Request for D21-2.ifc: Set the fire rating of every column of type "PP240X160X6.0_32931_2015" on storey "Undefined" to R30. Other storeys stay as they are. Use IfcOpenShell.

First a look at what the model holds.

```python
import ifcopenshell
import ifcopenshell.util.element

model = ifcopenshell.open("D21-2.ifc")
print(model.schema)
storey = next(s for s in model.by_type("IfcBuildingStorey") if s.Name == "Undefined")
columns = [e for e in ifcopenshell.util.element.get_decomposition(storey) if e.is_a("IfcColumn")]
seen = {}
for e in columns:
    element_type = ifcopenshell.util.element.get_type(e)
    key = (element_type.Name if element_type != e and element_type else None, ifcopenshell.util.element.get_pset(e, "Pset_ColumnCommon", "FireRating"))
    seen[key] = seen.get(key, 0) + 1
for (name, value), count in sorted(seen.items(), key=str):
    print(count, "x", name, "|", value)
```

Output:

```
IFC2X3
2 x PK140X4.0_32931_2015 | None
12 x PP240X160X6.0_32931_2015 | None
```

```python
import ifcopenshell
import ifcopenshell.api.pset
import ifcopenshell.util.element

model = ifcopenshell.open("D21-2.ifc")

storey = next(s for s in model.by_type("IfcBuildingStorey") if s.Name == "Undefined")
columns = [e for e in ifcopenshell.util.element.get_decomposition(storey) if e.is_a("IfcColumn")]

count = 0
for e in columns:
    element_type = ifcopenshell.util.element.get_type(e)
    if element_type in (None, e) or element_type.Name != "PP240X160X6.0_32931_2015":
        continue
    found = ifcopenshell.util.element.get_pset(e, "Pset_ColumnCommon", should_inherit=False)
    if found:
        pset = model.by_id(found["id"])
        if len(ifcopenshell.util.element.get_elements_by_pset(pset)) > 1:
            pset = ifcopenshell.api.pset.unshare_pset(model, products=[e], pset=pset)[0]
    else:
        pset = ifcopenshell.api.pset.add_pset(model, product=e, name="Pset_ColumnCommon")
    ifcopenshell.api.pset.edit_pset(model, pset=pset, properties={"FireRating": "R30"})
    count += 1

print(count, "columns updated")

model.write("D21-2_rev.ifc")
```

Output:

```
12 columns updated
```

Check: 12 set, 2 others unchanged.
